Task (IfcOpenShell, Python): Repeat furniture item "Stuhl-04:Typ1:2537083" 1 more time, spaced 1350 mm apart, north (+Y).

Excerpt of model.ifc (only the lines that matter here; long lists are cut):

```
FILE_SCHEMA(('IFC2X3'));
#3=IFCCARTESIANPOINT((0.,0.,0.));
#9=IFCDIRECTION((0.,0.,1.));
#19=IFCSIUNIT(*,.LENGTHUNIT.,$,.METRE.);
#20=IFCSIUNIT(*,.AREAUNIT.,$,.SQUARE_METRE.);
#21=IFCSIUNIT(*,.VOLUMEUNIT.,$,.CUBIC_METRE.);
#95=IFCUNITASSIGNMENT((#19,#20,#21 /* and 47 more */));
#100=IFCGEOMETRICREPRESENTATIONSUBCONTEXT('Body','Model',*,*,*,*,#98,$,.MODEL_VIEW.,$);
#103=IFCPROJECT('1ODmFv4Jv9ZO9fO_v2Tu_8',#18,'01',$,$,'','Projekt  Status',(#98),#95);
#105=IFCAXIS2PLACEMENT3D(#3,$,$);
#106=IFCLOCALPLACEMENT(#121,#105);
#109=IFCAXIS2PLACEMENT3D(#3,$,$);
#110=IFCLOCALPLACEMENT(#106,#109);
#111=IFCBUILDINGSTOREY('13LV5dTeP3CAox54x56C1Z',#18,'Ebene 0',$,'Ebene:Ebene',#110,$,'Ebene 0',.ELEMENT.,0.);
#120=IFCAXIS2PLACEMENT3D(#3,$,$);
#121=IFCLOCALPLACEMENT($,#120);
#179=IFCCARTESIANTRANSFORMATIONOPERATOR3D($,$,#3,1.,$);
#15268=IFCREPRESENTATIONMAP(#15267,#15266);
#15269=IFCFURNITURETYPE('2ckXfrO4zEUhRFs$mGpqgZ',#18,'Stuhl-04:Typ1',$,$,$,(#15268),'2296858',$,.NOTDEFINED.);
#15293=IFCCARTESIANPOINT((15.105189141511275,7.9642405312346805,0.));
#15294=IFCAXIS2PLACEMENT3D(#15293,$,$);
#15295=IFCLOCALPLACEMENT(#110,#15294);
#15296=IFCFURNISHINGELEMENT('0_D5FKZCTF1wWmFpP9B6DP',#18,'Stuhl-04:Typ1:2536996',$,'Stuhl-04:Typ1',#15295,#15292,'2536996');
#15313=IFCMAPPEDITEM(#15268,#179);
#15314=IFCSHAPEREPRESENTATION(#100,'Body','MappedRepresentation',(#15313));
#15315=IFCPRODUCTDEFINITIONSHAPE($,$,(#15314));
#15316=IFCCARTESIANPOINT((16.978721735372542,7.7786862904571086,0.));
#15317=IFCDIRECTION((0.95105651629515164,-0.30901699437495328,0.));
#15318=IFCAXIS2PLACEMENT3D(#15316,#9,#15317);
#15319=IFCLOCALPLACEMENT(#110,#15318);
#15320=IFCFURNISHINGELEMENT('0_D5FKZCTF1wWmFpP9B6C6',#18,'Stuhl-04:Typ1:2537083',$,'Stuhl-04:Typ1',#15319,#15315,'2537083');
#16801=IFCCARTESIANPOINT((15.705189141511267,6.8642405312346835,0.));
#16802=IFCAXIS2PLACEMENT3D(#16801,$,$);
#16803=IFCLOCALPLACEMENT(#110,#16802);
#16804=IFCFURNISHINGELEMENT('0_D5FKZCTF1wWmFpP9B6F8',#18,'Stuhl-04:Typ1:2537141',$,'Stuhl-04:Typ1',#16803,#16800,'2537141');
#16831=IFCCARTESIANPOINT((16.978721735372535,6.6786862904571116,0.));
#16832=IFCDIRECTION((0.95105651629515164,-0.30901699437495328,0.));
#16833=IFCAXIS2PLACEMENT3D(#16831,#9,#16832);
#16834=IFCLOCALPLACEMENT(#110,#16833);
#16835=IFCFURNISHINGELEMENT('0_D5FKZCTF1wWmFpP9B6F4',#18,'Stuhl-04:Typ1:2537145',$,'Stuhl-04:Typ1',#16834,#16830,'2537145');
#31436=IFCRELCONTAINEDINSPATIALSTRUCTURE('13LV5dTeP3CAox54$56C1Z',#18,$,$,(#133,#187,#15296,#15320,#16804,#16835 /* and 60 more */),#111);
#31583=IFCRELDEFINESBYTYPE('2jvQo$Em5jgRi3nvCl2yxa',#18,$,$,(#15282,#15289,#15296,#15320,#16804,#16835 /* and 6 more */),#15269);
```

```python
import numpy as np
import ifcopenshell
import ifcopenshell.api.geometry
import ifcopenshell.api.root
import ifcopenshell.util.element
import ifcopenshell.util.placement
import ifcopenshell.util.unit

model = ifcopenshell.open("model.ifc")
unit_scale = ifcopenshell.util.unit.calculate_unit_scale(model)

source = model.by_guid("0_D5FKZCTF1wWmFpP9B6C6")
base = ifcopenshell.util.placement.get_local_placement(source.ObjectPlacement)
step = np.array([0.0, 1.0, 0.0]) * 1.35 / unit_scale

for i in range(1, 2):
    copy = ifcopenshell.api.root.copy_class(model, product=source)
    copy.Representation = ifcopenshell.util.element.copy_deep(
        model, source.Representation, exclude=["IfcGeometricRepresentationContext", "IfcRepresentationMap"]
    )
    copy.Name = "Stuhl-04:Typ1"
    copy.Tag = None
    matrix = base.copy()
    matrix[:3, 3] += i * step
    print("added at", matrix[:3, 3].round(3) + 0.0)
    ifcopenshell.api.geometry.edit_object_placement(model, product=copy, matrix=matrix, is_si=False)

model.write("model_rev.ifc")
```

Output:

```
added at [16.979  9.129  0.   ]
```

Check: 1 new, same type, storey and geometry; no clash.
